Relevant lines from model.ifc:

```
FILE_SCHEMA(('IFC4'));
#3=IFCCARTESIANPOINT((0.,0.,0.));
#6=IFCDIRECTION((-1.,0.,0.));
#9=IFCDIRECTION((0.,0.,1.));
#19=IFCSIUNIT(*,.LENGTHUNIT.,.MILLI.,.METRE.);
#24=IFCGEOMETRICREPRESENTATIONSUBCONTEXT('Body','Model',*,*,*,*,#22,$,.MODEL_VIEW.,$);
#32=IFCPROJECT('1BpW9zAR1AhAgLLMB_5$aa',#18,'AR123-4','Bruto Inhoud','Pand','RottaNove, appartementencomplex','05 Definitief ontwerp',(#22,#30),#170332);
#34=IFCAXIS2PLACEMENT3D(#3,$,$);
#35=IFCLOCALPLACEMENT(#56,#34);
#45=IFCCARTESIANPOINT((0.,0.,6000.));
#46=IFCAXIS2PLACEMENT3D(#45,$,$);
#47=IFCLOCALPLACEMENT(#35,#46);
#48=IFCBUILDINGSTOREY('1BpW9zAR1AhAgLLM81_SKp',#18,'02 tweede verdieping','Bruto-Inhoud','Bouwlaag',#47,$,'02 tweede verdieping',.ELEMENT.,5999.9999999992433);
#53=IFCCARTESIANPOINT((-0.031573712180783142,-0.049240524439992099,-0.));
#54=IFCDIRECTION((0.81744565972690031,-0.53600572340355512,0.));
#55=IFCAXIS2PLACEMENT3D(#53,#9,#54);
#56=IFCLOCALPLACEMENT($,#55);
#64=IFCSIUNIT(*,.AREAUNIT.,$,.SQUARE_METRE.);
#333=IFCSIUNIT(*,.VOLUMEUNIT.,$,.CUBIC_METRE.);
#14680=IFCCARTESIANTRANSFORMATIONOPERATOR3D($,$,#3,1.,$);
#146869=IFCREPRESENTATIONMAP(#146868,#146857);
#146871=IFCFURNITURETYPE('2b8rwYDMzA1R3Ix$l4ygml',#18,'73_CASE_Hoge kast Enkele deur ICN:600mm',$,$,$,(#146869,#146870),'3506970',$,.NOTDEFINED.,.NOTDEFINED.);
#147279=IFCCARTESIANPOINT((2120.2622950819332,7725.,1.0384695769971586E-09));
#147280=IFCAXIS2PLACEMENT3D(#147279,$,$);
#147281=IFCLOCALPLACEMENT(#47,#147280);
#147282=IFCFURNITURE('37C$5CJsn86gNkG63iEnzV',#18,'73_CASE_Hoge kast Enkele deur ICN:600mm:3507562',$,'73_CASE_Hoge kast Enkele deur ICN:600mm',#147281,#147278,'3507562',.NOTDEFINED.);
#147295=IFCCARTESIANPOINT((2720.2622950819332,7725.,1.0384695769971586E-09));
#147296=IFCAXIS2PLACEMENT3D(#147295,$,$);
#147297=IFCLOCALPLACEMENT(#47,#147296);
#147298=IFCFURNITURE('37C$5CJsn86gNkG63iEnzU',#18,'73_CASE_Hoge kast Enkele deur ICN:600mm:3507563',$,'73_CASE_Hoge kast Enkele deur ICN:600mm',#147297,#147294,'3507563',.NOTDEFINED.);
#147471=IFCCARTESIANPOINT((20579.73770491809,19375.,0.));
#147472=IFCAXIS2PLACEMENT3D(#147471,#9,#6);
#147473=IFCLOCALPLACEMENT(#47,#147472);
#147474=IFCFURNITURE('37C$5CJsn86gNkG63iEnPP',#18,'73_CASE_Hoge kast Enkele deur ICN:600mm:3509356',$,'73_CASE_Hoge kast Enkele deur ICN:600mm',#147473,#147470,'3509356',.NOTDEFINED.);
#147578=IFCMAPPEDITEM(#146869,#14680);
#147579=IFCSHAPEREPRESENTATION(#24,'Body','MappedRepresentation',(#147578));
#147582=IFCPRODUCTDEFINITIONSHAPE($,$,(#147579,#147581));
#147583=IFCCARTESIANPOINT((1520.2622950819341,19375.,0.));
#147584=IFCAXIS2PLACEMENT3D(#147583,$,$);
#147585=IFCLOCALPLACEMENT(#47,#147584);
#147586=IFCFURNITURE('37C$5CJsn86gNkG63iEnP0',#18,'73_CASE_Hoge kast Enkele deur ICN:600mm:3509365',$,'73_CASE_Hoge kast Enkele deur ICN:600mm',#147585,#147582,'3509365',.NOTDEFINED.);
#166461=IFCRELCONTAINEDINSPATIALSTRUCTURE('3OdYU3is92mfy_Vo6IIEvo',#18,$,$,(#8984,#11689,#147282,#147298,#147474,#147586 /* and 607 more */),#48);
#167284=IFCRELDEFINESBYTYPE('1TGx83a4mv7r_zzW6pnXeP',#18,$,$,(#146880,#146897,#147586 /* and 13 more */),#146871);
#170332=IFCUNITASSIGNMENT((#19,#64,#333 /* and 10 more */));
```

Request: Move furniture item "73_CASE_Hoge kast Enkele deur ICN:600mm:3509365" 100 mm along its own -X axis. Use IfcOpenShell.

```python
import ifcopenshell
import ifcopenshell.api.geometry
import ifcopenshell.util.placement
import ifcopenshell.util.unit

model = ifcopenshell.open("model.ifc")
unit_scale = ifcopenshell.util.unit.calculate_unit_scale(model)

item = model.by_guid("37C$5CJsn86gNkG63iEnP0")
matrix = ifcopenshell.util.placement.get_local_placement(item.ObjectPlacement)
matrix[:3, 3] -= matrix[:3, 0] * 0.1 / unit_scale
ifcopenshell.api.geometry.edit_object_placement(model, product=item, matrix=matrix, is_si=False)

print(ifcopenshell.util.placement.get_local_placement(item.ObjectPlacement).round(3) + 0.0)

model.write("model_v2.ifc")
```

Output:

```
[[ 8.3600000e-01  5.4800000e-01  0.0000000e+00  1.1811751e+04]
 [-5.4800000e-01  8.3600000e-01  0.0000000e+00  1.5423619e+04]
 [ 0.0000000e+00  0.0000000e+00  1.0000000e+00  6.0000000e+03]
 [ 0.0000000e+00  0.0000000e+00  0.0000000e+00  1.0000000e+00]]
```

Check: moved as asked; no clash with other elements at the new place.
